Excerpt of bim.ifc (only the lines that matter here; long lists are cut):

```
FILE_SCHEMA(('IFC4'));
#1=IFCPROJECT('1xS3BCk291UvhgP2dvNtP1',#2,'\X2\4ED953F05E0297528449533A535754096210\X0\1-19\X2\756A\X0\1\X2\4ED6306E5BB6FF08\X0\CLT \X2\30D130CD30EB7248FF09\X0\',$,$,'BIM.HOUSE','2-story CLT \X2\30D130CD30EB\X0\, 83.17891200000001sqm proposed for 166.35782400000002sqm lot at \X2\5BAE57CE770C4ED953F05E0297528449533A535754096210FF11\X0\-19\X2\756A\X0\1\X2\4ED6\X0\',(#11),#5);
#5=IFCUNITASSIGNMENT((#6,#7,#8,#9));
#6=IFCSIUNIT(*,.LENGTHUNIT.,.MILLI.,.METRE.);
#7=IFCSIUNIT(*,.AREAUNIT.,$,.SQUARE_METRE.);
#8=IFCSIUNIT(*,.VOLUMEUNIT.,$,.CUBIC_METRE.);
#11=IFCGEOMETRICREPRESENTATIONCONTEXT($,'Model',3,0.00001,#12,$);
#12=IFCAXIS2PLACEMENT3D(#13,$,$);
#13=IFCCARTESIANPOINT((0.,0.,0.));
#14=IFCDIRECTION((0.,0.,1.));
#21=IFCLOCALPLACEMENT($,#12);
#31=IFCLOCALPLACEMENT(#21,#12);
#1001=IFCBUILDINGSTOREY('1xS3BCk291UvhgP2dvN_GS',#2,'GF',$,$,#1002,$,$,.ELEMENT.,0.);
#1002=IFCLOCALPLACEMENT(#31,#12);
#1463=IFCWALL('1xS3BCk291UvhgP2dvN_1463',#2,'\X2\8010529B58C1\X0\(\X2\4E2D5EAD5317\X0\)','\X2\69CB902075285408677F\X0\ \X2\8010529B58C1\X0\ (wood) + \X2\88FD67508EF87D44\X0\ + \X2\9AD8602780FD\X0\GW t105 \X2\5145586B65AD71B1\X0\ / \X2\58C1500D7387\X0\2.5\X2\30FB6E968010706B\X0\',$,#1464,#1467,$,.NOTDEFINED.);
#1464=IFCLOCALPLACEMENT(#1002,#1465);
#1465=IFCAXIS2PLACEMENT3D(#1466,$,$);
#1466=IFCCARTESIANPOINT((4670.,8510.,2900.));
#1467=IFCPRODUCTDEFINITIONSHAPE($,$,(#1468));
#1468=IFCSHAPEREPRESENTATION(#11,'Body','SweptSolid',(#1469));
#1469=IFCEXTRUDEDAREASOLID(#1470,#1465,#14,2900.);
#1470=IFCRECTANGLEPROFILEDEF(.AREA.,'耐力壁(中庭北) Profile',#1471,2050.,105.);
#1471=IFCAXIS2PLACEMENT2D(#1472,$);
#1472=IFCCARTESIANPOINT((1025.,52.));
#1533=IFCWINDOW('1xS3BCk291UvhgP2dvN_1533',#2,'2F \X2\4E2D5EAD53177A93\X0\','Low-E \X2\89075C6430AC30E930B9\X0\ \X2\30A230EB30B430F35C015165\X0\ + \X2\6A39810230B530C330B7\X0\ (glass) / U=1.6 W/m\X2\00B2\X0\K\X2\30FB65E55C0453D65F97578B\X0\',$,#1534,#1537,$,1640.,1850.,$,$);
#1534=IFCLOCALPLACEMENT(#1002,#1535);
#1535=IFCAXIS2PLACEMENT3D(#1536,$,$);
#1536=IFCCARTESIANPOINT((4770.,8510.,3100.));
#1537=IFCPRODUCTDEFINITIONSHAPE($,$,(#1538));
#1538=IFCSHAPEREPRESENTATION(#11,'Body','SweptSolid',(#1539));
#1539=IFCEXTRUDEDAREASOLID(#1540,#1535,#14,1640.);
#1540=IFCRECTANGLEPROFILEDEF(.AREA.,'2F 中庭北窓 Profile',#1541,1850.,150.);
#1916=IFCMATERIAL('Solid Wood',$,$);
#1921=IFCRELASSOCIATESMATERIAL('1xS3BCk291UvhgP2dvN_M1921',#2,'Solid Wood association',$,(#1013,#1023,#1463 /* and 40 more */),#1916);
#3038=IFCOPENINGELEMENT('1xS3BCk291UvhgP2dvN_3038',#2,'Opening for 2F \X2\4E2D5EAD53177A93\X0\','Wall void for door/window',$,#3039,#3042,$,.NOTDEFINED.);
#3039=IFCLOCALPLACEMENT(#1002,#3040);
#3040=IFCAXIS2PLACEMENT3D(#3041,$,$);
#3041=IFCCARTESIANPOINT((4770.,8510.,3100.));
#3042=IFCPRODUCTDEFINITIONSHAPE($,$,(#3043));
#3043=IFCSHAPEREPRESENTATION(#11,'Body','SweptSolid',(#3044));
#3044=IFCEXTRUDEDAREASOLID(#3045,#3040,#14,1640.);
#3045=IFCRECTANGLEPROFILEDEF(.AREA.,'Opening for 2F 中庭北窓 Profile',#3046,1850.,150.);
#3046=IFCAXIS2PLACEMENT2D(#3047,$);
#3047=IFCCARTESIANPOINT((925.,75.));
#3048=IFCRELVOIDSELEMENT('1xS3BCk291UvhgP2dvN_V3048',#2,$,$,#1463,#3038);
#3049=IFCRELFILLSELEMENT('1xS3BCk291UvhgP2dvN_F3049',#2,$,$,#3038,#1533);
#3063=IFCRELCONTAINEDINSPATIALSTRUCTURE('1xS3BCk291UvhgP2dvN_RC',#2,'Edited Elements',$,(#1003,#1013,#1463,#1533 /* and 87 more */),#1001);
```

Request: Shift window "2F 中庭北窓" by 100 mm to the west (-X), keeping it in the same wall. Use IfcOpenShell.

```python
import ifcopenshell
import ifcopenshell.api.geometry
import ifcopenshell.util.placement
import ifcopenshell.util.unit

model = ifcopenshell.open("bim.ifc")
unit_scale = ifcopenshell.util.unit.calculate_unit_scale(model)

window = model.by_guid("1xS3BCk291UvhgP2dvN_1533")
opening = window.FillsVoids[0].RelatingOpeningElement
wall = opening.VoidsElements[0].RelatingBuildingElement

wall_matrix = ifcopenshell.util.placement.get_local_placement(wall.ObjectPlacement)
shift = wall_matrix[:3, 0] * -0.1 / unit_scale
before = ifcopenshell.util.placement.get_local_placement(window.ObjectPlacement)[:3, 3].copy()

# The window is not placed relative to its opening, so move both.
for product in (opening, window):
    matrix = ifcopenshell.util.placement.get_local_placement(product.ObjectPlacement)
    matrix[:3, 3] += shift
    ifcopenshell.api.geometry.edit_object_placement(model, product=product, matrix=matrix, is_si=False)

after = ifcopenshell.util.placement.get_local_placement(window.ObjectPlacement)[:3, 3]
print("window moved by", (after - before).round(3) + 0.0)

model.write("bim-out.ifc")
```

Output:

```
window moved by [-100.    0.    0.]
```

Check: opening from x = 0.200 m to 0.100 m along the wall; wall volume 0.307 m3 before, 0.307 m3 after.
